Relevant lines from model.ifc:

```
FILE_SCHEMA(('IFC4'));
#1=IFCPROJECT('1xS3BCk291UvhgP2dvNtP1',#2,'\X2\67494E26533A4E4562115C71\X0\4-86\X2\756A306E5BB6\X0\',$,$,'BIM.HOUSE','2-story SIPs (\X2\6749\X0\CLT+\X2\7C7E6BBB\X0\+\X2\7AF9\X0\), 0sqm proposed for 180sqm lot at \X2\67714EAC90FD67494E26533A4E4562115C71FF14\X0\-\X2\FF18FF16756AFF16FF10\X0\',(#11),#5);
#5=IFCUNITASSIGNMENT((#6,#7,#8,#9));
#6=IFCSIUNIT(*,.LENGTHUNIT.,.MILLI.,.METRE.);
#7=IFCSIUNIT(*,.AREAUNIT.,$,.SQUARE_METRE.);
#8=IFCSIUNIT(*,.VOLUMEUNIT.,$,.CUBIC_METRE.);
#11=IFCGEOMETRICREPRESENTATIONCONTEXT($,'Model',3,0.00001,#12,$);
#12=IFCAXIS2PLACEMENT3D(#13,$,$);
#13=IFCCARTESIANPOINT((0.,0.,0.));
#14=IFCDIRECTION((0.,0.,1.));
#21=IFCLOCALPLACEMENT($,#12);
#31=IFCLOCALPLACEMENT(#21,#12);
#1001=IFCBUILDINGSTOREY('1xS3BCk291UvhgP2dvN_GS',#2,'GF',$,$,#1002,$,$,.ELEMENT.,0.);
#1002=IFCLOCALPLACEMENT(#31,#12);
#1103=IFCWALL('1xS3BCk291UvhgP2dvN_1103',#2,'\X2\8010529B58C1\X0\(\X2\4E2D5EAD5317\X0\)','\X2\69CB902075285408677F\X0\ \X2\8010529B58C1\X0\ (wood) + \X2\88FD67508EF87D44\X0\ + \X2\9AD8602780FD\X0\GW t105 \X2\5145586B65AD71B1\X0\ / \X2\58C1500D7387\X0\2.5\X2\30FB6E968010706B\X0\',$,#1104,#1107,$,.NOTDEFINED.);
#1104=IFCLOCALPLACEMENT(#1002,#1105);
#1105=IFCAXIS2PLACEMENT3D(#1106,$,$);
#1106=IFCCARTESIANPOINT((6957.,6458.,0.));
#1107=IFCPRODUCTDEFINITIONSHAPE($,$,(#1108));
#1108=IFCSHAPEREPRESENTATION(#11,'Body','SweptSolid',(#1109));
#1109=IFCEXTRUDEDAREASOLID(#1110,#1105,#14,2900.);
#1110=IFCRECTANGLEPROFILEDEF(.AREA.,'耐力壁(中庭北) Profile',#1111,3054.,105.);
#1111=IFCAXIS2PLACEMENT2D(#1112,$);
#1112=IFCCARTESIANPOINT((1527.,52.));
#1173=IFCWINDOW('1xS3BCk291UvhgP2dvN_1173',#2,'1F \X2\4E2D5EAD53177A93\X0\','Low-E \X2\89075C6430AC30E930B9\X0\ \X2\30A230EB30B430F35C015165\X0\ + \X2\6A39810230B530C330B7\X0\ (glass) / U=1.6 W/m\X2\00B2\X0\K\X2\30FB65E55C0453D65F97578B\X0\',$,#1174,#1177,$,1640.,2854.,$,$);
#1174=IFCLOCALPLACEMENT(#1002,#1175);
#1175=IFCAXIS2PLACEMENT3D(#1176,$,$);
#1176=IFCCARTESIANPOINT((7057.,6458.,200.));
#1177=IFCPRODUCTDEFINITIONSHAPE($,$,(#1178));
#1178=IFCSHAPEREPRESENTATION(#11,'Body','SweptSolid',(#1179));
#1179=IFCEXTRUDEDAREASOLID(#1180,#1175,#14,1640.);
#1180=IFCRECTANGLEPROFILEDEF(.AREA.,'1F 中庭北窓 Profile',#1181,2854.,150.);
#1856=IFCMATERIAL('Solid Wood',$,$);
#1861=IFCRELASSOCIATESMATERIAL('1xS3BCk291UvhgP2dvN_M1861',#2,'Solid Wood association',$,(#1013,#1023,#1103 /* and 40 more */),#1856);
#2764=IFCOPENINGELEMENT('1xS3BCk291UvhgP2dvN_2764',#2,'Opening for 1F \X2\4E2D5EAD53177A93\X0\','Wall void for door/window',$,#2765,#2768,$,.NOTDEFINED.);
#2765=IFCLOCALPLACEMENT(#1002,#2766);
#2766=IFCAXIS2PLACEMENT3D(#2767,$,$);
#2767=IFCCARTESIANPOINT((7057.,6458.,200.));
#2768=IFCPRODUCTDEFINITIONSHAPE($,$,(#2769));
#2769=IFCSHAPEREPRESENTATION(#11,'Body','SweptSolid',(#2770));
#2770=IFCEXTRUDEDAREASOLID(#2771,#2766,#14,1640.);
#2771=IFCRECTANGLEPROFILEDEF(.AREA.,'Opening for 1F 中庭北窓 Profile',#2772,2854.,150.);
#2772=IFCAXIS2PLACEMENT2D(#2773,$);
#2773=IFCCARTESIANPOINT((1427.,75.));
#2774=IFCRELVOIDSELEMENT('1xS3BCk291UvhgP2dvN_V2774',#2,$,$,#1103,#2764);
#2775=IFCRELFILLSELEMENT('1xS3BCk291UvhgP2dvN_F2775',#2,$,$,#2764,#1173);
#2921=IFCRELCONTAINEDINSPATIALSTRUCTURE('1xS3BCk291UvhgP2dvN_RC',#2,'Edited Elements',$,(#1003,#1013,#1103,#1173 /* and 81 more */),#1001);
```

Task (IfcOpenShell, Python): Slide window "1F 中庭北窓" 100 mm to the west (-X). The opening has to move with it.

```python
import ifcopenshell
import ifcopenshell.api.geometry
import ifcopenshell.util.placement
import ifcopenshell.util.unit

model = ifcopenshell.open("model.ifc")
unit_scale = ifcopenshell.util.unit.calculate_unit_scale(model)

window = model.by_guid("1xS3BCk291UvhgP2dvN_1173")
opening = window.FillsVoids[0].RelatingOpeningElement
wall = opening.VoidsElements[0].RelatingBuildingElement

wall_matrix = ifcopenshell.util.placement.get_local_placement(wall.ObjectPlacement)
shift = wall_matrix[:3, 0] * -0.1 / unit_scale
before = ifcopenshell.util.placement.get_local_placement(window.ObjectPlacement)[:3, 3].copy()

# The window is not placed relative to its opening, so move both.
for product in (opening, window):
    matrix = ifcopenshell.util.placement.get_local_placement(product.ObjectPlacement)
    matrix[:3, 3] += shift
    ifcopenshell.api.geometry.edit_object_placement(model, product=product, matrix=matrix, is_si=False)

after = ifcopenshell.util.placement.get_local_placement(window.ObjectPlacement)[:3, 3]
print("window moved by", (after - before).round(3) + 0.0)

model.write("model_v2.ifc")
```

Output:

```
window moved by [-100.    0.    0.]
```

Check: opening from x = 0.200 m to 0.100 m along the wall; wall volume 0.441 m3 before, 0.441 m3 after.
